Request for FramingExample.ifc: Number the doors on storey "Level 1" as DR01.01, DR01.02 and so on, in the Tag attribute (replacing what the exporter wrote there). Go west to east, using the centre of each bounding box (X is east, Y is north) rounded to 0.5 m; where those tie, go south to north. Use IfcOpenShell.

First a look at what the model holds.

```python
import ifcopenshell
import ifcopenshell.util.element
import ifcopenshell.util.placement

model = ifcopenshell.open("FramingExample.ifc")
print(model.schema)
storey = next(s for s in model.by_type("IfcBuildingStorey") if s.Name == "Level 1")
doors = [e for e in ifcopenshell.util.element.get_decomposition(storey) if e.is_a("IfcDoor")]
for e in sorted(doors, key=lambda e: e.id()):
    origin = ifcopenshell.util.placement.get_local_placement(e.ObjectPlacement)[:3, 3]
    print(e.id(), e.Tag, e.Name, origin.round(2) + 0.0, sep=" | ")
```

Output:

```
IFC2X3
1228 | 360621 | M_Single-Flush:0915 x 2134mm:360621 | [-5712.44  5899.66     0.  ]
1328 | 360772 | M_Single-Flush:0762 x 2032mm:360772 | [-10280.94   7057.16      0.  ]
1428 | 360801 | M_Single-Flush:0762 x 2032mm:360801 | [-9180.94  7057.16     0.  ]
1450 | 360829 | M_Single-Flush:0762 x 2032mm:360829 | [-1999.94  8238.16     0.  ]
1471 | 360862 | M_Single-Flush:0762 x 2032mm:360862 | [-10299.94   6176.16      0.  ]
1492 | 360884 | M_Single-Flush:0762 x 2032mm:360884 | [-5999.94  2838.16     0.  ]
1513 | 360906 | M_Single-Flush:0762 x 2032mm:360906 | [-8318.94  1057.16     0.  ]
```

```python
import ifcopenshell
import ifcopenshell.geom
import ifcopenshell.util.element
import ifcopenshell.util.shape

model = ifcopenshell.open("FramingExample.ifc")
settings = ifcopenshell.geom.settings()
settings.set("use-world-coords", True)


def centre(element):
    shape = ifcopenshell.geom.create_shape(settings, element)
    return ifcopenshell.util.shape.get_bbox_centroid(shape.geometry)


storey = next(s for s in model.by_type("IfcBuildingStorey") if s.Name == "Level 1")
doors = [e for e in ifcopenshell.util.element.get_decomposition(storey) if e.is_a("IfcDoor")]

# Insertion points can sit at a corner or the storey origin, so sort by the geometry (in metres).
centres = {e: centre(e) for e in doors}
doors.sort(key=lambda e: (round(centres[e][0] / 0.5), centres[e][1]))

for i, e in enumerate(doors, start=1):
    number = f"DR01.{i:02d}"
    e.Tag = number
    print(e.id(), number)

model.write("FramingExample_updated.ifc")
```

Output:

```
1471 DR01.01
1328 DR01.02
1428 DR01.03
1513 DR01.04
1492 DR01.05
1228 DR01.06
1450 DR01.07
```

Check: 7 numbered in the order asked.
